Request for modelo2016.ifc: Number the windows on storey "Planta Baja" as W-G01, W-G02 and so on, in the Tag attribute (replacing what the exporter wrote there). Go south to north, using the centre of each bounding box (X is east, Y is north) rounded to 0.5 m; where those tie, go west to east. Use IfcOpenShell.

First a look at what the model holds.

```python
import ifcopenshell
import ifcopenshell.util.element
import ifcopenshell.util.placement

model = ifcopenshell.open("modelo2016.ifc")
print(model.schema)
storey = next(s for s in model.by_type("IfcBuildingStorey") if s.Name == "Planta Baja")
windows = [e for e in ifcopenshell.util.element.get_decomposition(storey) if e.is_a("IfcWindow")]
for e in sorted(windows, key=lambda e: e.id()):
    origin = ifcopenshell.util.placement.get_local_placement(e.ObjectPlacement)[:3, 3]
    print(e.id(), e.Tag, e.Name, origin.round(2) + 0.0, sep=" | ")
```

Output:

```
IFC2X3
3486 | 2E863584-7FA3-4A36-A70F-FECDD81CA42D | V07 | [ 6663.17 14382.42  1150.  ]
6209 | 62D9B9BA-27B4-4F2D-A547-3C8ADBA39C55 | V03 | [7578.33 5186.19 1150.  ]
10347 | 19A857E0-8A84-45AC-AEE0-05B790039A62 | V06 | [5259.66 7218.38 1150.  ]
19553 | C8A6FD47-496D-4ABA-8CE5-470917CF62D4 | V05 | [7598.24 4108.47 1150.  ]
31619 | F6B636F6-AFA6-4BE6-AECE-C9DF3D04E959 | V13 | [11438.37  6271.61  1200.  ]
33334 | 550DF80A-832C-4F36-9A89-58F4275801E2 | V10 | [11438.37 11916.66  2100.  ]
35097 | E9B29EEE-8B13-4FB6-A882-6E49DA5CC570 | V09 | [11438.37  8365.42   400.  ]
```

```python
import ifcopenshell
import ifcopenshell.geom
import ifcopenshell.util.element
import ifcopenshell.util.shape

model = ifcopenshell.open("modelo2016.ifc")
settings = ifcopenshell.geom.settings()
settings.set("use-world-coords", True)


def centre(element):
    shape = ifcopenshell.geom.create_shape(settings, element)
    return ifcopenshell.util.shape.get_bbox_centroid(shape.geometry)


storey = next(s for s in model.by_type("IfcBuildingStorey") if s.Name == "Planta Baja")
windows = [e for e in ifcopenshell.util.element.get_decomposition(storey) if e.is_a("IfcWindow")]

# Insertion points can sit at a corner or the storey origin, so sort by the geometry (in metres).
centres = {e: centre(e) for e in windows}
windows.sort(key=lambda e: (round(centres[e][1] / 0.5), centres[e][0]))

for i, e in enumerate(windows, start=1):
    number = f"W-G{i:02d}"
    e.Tag = number
    print(e.id(), number)

model.write("modelo2016_rev.ifc")
```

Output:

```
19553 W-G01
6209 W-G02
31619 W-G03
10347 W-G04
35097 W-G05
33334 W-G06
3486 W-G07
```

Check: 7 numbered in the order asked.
